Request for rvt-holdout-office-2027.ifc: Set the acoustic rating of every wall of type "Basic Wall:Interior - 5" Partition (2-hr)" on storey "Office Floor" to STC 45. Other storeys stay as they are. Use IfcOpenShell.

First a look at what the model holds.

```python
import ifcopenshell
import ifcopenshell.util.element

model = ifcopenshell.open("rvt-holdout-office-2027.ifc")
print(model.schema)
storey = next(s for s in model.by_type("IfcBuildingStorey") if s.Name == "Office Floor")
walls = [e for e in ifcopenshell.util.element.get_decomposition(storey) if e.is_a("IfcWall")]
seen = {}
for e in walls:
    element_type = ifcopenshell.util.element.get_type(e)
    key = (element_type.Name if element_type != e and element_type else None, ifcopenshell.util.element.get_pset(e, "Pset_WallCommon", "AcousticRating"))
    seen[key] = seen.get(key, 0) + 1
for (name, value), count in sorted(seen.items(), key=str):
    print(count, "x", name, "|", value)
```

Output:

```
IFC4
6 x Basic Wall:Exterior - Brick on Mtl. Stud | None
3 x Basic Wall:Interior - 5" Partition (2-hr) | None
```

```python
import ifcopenshell
import ifcopenshell.api.pset
import ifcopenshell.util.element

model = ifcopenshell.open("rvt-holdout-office-2027.ifc")

storey = next(s for s in model.by_type("IfcBuildingStorey") if s.Name == "Office Floor")
walls = [e for e in ifcopenshell.util.element.get_decomposition(storey) if e.is_a("IfcWall")]

count = 0
for e in walls:
    element_type = ifcopenshell.util.element.get_type(e)
    if element_type in (None, e) or element_type.Name != 'Basic Wall:Interior - 5" Partition (2-hr)':
        continue
    # add_pset returns the element's existing set when there is one.
    pset = ifcopenshell.api.pset.add_pset(model, product=e, name="Pset_WallCommon")
    ifcopenshell.api.pset.edit_pset(model, pset=pset, properties={"AcousticRating": "STC 45"})
    count += 1

print(count, "walls updated")

model.write("rvt-holdout-office-2027_edited.ifc")
```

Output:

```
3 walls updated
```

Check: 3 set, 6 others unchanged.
